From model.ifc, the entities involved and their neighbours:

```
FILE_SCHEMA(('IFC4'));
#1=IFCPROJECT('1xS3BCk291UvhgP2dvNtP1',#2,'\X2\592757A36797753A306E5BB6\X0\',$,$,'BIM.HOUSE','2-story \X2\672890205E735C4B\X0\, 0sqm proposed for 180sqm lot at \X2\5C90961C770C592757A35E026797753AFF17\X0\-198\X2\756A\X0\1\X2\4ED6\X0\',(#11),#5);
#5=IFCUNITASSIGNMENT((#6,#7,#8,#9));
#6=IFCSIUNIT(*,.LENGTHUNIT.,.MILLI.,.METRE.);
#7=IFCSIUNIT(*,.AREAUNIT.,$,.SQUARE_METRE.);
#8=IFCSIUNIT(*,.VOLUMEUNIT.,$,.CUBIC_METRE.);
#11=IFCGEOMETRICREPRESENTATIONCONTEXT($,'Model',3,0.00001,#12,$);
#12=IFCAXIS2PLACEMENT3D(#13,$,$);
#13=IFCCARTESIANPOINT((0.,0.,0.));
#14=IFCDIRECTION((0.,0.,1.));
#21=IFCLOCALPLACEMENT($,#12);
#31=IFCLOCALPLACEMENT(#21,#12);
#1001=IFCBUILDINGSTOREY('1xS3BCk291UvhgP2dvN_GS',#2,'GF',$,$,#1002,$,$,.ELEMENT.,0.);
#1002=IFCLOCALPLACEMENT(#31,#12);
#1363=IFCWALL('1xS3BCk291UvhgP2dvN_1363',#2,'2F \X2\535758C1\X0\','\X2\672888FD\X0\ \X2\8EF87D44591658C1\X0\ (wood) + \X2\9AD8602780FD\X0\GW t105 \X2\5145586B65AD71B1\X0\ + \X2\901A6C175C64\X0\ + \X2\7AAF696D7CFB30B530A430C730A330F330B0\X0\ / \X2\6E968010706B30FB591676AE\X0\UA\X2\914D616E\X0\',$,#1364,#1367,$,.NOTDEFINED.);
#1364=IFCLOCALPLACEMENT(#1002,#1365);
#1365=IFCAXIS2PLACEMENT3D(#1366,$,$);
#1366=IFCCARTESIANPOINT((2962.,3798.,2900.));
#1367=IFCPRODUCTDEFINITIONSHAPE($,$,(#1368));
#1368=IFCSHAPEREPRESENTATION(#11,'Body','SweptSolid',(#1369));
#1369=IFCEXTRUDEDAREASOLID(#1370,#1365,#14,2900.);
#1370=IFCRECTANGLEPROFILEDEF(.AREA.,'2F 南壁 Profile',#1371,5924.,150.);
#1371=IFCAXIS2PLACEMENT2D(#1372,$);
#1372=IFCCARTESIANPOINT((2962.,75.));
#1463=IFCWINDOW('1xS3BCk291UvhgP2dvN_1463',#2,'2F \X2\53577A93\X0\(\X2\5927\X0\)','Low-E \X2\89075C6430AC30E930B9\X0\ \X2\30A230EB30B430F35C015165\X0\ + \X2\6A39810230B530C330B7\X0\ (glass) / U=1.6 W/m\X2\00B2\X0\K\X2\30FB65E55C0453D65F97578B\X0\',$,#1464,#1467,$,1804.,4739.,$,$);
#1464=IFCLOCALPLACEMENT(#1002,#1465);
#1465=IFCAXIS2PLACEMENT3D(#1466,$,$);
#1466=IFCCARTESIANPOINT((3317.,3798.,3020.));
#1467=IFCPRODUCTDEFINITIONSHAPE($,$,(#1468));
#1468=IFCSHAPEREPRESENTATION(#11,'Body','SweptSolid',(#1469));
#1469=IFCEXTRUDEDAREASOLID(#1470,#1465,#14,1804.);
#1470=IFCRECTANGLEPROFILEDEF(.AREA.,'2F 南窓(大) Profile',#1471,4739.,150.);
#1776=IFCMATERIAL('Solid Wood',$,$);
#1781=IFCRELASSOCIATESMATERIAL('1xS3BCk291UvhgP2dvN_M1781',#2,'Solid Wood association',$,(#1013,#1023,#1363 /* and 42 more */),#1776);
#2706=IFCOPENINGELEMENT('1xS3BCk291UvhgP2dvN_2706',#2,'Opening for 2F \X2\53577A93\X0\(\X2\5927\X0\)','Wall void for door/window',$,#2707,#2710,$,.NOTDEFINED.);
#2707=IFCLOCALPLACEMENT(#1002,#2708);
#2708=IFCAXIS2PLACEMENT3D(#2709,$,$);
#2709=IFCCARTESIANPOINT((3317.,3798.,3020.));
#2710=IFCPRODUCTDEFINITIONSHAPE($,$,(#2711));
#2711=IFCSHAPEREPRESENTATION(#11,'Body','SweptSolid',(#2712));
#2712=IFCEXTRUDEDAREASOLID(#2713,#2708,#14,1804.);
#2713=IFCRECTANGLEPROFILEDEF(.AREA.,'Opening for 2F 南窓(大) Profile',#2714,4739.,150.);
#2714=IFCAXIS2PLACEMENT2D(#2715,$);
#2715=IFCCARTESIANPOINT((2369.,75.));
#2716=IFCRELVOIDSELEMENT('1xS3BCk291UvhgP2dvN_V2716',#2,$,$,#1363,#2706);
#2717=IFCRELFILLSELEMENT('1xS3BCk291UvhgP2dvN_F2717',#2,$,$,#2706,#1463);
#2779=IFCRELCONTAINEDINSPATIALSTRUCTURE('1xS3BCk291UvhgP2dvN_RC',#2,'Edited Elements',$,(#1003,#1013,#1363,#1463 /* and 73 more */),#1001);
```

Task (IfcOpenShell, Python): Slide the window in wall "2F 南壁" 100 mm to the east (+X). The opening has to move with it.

```python
import ifcopenshell
import ifcopenshell.api.geometry
import ifcopenshell.util.placement

model = ifcopenshell.open("model.ifc")

window = model.by_id(1463)
opening = window.FillsVoids[0].RelatingOpeningElement
wall = opening.VoidsElements[0].RelatingBuildingElement

wall_matrix = ifcopenshell.util.placement.get_local_placement(wall.ObjectPlacement)
shift = wall_matrix[:3, 0] * 100.0
before = ifcopenshell.util.placement.get_local_placement(window.ObjectPlacement)[:3, 3].copy()

# The window is not placed relative to its opening, so move both.
for product in (opening, window):
    matrix = ifcopenshell.util.placement.get_local_placement(product.ObjectPlacement)
    matrix[:3, 3] += shift
    ifcopenshell.api.geometry.edit_object_placement(model, product=product, matrix=matrix, is_si=False)

after = ifcopenshell.util.placement.get_local_placement(window.ObjectPlacement)[:3, 3]
print("window moved by", (after - before).round(3) + 0.0)

model.write("model_updated.ifc")
```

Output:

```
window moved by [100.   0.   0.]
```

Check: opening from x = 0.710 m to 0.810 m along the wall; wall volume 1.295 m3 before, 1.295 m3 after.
